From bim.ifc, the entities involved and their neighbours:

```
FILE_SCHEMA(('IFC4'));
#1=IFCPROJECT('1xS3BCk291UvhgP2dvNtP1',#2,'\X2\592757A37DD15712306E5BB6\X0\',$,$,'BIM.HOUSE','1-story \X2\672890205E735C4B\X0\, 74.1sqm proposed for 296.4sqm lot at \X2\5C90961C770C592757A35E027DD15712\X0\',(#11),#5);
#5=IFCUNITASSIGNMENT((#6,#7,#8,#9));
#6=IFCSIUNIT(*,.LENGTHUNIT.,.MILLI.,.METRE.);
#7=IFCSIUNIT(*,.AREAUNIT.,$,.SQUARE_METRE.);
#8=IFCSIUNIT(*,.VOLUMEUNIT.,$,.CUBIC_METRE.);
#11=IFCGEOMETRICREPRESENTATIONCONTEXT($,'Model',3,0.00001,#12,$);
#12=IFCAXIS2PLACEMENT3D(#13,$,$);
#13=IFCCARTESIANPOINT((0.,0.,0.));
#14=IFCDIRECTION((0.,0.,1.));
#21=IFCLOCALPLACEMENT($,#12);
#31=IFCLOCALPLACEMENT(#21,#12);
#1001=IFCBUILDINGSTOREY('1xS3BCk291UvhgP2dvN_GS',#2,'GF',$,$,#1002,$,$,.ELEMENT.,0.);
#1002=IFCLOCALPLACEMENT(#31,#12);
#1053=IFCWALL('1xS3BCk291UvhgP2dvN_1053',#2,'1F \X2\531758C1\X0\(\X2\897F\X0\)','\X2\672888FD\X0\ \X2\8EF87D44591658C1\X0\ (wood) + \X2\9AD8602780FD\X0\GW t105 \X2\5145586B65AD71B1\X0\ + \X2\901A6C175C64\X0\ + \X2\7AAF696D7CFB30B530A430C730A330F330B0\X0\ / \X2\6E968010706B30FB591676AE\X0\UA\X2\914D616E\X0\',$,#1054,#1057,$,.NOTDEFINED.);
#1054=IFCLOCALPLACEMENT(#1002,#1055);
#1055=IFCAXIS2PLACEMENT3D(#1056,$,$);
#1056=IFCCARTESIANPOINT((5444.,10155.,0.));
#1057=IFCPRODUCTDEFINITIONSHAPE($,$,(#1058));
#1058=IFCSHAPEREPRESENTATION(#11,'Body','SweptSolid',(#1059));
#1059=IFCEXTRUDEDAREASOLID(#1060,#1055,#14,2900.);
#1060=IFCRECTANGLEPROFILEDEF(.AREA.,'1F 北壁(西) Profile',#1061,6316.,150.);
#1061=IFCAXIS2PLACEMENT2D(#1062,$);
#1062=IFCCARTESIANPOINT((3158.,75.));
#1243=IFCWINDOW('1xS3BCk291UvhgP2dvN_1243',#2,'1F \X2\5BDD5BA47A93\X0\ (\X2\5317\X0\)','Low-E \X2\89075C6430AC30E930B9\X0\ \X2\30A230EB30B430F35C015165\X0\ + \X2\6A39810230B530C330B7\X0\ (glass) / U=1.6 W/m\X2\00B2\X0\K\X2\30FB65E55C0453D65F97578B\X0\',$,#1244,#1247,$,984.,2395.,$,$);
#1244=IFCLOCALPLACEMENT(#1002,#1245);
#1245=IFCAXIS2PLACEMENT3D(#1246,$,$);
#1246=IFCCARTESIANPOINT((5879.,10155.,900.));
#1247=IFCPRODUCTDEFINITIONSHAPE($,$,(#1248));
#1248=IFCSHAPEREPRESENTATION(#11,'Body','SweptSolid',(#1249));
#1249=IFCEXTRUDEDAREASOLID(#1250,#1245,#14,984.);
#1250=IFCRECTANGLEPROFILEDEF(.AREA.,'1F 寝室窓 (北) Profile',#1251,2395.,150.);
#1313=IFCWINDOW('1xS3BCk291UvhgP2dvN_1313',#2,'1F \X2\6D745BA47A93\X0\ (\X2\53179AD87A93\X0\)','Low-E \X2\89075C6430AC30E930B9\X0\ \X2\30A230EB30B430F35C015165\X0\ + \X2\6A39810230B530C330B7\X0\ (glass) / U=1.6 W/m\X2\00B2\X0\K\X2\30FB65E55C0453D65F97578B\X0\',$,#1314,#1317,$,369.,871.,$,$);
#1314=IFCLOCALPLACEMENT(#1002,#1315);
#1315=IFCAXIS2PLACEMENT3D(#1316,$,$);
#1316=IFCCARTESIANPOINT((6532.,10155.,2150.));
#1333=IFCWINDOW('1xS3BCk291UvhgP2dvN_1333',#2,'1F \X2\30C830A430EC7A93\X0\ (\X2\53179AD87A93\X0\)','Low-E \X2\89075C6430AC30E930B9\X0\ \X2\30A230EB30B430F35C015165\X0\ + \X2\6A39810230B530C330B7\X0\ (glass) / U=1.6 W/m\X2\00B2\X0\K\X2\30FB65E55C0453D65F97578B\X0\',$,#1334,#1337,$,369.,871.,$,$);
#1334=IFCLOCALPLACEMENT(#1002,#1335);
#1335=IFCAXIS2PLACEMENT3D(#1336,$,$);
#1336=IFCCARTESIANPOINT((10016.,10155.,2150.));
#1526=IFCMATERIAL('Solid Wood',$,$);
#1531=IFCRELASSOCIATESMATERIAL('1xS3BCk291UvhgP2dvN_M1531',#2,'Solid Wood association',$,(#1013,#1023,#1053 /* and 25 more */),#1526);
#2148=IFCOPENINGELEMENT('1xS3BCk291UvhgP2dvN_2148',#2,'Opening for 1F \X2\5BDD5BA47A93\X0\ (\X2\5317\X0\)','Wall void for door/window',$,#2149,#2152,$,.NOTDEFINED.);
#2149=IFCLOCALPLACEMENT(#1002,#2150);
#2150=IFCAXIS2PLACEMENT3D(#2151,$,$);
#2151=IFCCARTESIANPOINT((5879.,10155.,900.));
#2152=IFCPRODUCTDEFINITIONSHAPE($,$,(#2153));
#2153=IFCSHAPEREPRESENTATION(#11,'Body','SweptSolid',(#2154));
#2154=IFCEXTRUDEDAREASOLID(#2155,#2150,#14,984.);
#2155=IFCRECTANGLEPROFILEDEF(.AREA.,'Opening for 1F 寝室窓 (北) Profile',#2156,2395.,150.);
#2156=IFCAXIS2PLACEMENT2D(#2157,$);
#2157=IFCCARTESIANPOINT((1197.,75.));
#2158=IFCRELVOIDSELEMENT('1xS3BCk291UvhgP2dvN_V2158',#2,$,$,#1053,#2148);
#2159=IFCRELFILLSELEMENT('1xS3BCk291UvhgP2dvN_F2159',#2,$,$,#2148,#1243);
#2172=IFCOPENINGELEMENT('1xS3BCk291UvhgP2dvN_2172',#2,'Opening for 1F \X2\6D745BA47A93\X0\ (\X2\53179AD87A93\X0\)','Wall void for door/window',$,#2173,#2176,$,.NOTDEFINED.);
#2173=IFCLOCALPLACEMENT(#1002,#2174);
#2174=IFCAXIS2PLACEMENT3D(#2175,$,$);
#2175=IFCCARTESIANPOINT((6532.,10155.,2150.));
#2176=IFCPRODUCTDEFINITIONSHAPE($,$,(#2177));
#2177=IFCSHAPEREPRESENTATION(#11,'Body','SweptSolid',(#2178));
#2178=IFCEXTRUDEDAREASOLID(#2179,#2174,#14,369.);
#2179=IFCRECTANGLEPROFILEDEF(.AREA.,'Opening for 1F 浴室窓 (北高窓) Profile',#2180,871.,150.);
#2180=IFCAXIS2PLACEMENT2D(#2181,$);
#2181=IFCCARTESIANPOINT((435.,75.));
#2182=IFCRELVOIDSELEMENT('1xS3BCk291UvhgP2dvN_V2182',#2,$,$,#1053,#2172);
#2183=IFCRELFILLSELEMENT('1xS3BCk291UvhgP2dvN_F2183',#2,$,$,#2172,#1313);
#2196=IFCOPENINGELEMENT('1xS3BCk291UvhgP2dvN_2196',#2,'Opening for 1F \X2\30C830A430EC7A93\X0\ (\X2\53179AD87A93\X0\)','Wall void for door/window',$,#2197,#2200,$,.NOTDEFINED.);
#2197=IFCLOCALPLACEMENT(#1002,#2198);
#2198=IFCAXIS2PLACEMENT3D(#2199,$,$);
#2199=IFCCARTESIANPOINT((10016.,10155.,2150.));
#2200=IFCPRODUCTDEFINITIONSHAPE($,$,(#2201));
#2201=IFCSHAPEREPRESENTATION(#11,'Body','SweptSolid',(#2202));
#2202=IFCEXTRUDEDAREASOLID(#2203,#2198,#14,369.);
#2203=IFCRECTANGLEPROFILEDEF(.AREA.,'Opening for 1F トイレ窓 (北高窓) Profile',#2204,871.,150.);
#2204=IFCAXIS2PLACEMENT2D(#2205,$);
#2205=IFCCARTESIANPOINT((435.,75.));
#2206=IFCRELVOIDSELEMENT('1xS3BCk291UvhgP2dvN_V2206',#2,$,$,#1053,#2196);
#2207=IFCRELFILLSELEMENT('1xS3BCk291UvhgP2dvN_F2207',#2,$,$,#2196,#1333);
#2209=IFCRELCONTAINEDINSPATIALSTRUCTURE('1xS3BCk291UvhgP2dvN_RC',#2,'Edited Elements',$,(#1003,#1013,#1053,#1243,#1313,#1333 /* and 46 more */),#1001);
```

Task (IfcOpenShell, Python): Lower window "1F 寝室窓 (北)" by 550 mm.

```python
import numpy as np
import ifcopenshell
import ifcopenshell.api.geometry
import ifcopenshell.util.placement
import ifcopenshell.util.unit

model = ifcopenshell.open("bim.ifc")
unit_scale = ifcopenshell.util.unit.calculate_unit_scale(model)

window = model.by_guid("1xS3BCk291UvhgP2dvN_1243")
opening = window.FillsVoids[0].RelatingOpeningElement
dz = -0.55 / unit_scale

shift = np.array([0.0, 0.0, dz])
# The window is not placed relative to its opening, so move both.
for product in (opening, window):
    matrix = ifcopenshell.util.placement.get_local_placement(product.ObjectPlacement)
    matrix[:3, 3] += shift
    ifcopenshell.api.geometry.edit_object_placement(model, product=product, matrix=matrix, is_si=False)

print(f"moved by {dz * unit_scale:+.3f} m")

model.write("bim_rev.ifc")
```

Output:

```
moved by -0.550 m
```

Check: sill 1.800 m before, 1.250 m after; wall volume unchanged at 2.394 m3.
